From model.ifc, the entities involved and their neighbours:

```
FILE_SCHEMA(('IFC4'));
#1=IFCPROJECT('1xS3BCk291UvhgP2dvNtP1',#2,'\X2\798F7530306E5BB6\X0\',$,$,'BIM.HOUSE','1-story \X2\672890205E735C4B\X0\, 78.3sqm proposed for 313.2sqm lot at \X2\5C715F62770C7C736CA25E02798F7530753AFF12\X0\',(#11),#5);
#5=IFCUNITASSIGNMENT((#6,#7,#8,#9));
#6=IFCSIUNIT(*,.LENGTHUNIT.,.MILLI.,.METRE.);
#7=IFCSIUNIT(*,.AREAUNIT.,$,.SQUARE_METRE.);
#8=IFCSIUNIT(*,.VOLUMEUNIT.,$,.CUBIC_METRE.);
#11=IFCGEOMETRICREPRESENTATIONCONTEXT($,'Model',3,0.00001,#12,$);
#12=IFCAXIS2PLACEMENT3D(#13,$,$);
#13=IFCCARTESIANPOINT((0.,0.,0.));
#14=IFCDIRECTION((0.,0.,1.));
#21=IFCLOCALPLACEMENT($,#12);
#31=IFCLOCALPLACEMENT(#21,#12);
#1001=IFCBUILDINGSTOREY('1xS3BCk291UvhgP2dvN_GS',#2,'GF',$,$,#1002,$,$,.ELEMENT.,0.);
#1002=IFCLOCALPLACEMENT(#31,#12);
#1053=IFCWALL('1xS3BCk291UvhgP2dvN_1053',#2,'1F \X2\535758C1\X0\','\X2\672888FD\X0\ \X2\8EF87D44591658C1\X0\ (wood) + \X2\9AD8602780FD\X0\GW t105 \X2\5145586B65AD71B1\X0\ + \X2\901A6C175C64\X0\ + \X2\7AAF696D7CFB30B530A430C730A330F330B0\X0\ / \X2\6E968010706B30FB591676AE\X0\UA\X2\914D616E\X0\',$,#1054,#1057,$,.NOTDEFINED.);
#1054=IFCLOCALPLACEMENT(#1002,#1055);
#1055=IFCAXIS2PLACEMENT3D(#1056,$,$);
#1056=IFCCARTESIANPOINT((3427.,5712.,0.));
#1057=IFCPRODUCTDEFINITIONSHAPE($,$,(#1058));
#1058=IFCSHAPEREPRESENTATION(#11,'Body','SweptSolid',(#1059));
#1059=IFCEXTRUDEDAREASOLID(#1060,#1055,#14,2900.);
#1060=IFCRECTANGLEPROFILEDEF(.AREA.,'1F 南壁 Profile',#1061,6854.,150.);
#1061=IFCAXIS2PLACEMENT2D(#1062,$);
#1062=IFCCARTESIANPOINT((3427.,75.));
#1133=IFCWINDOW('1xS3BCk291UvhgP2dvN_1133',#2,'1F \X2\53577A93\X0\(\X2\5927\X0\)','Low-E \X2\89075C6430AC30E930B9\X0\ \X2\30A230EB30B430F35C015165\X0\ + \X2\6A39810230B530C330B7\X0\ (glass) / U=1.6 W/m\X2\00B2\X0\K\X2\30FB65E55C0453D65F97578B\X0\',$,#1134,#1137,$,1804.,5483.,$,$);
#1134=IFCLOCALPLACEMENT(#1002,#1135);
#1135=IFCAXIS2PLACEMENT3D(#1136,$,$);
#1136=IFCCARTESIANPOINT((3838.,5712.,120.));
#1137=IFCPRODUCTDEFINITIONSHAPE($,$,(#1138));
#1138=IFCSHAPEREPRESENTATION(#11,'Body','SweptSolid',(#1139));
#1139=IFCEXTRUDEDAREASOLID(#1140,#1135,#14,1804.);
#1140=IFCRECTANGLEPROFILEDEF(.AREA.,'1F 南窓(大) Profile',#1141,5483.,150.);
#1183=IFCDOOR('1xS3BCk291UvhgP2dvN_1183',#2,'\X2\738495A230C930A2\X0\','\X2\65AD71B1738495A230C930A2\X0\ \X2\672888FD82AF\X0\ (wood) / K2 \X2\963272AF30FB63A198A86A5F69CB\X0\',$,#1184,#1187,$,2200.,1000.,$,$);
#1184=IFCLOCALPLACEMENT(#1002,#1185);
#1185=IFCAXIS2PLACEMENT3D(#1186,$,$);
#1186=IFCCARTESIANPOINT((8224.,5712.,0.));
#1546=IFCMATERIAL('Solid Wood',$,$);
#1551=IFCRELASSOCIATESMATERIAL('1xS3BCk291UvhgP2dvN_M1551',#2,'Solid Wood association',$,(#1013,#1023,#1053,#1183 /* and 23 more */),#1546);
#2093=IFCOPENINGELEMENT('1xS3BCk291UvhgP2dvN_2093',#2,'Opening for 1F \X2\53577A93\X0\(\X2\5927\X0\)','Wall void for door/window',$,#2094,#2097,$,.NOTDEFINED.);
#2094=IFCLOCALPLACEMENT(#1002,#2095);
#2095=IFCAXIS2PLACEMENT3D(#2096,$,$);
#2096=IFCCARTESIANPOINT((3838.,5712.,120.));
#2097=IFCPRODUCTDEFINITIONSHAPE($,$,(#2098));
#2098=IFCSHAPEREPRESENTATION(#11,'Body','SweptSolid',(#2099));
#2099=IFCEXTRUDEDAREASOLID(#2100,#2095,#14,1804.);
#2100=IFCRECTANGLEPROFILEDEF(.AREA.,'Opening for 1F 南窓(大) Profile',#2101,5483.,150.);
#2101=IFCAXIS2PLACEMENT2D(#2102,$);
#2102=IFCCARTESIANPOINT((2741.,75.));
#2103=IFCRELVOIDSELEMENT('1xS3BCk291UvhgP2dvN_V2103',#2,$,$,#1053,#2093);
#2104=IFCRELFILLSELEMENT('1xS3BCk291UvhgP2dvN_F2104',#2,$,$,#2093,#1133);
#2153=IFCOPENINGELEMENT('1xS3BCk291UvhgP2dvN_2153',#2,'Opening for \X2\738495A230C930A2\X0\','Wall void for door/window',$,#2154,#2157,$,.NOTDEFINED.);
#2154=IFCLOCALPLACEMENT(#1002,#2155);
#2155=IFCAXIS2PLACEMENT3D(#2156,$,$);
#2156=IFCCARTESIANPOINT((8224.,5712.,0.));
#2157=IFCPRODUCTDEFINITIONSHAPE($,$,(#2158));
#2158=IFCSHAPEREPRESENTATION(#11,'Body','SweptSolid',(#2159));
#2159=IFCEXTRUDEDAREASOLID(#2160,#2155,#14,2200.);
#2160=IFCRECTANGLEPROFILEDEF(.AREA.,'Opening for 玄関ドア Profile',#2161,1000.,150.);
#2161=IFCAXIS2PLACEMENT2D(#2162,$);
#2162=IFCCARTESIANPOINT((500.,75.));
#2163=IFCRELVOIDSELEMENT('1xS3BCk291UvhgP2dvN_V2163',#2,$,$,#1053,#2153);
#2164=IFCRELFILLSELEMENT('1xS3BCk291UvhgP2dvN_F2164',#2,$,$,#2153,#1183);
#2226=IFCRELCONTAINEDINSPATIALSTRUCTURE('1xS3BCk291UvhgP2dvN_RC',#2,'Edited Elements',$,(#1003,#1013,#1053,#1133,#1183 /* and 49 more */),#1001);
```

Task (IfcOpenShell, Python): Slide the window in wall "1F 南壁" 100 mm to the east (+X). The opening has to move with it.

```python
import ifcopenshell
import ifcopenshell.api.geometry
import ifcopenshell.util.placement

model = ifcopenshell.open("model.ifc")

window = model.by_guid("1xS3BCk291UvhgP2dvN_1133")
opening = window.FillsVoids[0].RelatingOpeningElement
wall = opening.VoidsElements[0].RelatingBuildingElement

wall_matrix = ifcopenshell.util.placement.get_local_placement(wall.ObjectPlacement)
shift = wall_matrix[:3, 0] * 100.0
before = ifcopenshell.util.placement.get_local_placement(window.ObjectPlacement)[:3, 3].copy()

# The window is not placed relative to its opening, so move both.
for product in (opening, window):
    matrix = ifcopenshell.util.placement.get_local_placement(product.ObjectPlacement)
    matrix[:3, 3] += shift
    ifcopenshell.api.geometry.edit_object_placement(model, product=product, matrix=matrix, is_si=False)

after = ifcopenshell.util.placement.get_local_placement(window.ObjectPlacement)[:3, 3]
print("window moved by", (after - before).round(3) + 0.0)

model.write("model-out.ifc")
```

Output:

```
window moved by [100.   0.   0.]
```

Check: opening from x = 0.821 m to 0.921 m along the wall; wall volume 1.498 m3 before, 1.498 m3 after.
